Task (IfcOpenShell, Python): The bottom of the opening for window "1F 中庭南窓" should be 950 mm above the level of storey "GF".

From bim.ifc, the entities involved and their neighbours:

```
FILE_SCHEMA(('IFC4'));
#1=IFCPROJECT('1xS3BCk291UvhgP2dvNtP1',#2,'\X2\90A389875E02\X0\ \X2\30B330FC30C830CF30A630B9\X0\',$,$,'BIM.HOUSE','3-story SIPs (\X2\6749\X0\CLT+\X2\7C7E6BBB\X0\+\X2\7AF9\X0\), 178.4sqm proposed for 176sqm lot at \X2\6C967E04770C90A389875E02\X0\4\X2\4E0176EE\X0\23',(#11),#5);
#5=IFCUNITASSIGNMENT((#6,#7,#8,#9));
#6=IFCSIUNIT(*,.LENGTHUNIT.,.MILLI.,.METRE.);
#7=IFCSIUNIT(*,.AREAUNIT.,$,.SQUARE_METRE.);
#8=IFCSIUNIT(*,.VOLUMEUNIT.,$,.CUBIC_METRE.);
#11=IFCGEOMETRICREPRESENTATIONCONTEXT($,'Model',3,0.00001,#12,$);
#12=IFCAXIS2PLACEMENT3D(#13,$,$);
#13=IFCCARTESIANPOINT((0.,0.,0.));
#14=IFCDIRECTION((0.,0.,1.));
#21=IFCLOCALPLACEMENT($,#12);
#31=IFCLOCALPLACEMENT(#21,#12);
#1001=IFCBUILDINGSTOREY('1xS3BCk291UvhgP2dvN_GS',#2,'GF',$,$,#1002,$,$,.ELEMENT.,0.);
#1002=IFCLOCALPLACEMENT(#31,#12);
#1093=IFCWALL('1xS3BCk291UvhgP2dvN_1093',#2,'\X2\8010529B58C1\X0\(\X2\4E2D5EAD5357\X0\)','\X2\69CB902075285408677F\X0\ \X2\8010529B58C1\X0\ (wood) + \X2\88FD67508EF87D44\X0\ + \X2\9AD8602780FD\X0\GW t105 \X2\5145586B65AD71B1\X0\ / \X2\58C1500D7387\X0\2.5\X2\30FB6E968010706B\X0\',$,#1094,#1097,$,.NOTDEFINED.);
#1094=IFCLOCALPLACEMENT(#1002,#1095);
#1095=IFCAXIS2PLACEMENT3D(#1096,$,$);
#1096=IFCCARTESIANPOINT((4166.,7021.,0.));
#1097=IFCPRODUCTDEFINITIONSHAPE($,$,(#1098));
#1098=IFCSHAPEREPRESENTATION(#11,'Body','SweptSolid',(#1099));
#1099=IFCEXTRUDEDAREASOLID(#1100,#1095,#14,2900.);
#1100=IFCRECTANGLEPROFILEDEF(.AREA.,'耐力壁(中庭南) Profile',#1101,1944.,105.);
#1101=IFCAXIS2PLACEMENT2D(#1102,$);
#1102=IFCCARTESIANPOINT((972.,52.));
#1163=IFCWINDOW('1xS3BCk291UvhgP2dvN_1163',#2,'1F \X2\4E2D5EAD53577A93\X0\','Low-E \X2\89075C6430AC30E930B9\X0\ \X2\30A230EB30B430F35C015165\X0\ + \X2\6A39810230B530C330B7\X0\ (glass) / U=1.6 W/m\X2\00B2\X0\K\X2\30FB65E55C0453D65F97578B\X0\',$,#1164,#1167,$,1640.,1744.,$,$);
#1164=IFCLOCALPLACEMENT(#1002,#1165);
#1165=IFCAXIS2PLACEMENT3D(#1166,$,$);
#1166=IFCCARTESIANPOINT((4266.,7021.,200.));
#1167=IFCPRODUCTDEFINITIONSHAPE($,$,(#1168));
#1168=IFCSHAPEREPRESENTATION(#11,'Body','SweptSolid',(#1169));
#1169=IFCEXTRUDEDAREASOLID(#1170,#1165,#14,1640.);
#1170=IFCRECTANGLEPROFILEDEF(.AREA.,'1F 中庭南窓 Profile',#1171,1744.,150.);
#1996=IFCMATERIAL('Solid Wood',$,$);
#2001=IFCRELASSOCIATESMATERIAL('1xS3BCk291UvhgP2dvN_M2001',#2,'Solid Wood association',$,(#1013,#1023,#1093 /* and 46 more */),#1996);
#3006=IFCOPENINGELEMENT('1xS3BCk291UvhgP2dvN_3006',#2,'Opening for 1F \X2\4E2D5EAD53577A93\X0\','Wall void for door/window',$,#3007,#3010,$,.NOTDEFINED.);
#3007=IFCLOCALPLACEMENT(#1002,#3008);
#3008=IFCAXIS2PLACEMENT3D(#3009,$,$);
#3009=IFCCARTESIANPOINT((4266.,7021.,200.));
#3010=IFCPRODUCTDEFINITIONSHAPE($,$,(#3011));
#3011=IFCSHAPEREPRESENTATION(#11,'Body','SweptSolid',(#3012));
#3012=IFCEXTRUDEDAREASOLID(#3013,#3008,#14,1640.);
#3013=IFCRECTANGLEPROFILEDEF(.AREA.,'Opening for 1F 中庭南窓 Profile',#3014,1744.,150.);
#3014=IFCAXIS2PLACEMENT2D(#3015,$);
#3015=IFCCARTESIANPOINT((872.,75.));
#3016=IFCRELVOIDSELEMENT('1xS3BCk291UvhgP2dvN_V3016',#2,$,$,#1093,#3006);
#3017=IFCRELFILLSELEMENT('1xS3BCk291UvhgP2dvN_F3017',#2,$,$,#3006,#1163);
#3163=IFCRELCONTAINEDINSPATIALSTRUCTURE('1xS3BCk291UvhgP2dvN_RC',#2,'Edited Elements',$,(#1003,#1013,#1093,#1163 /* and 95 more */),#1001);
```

```python
import numpy as np
import ifcopenshell
import ifcopenshell.api.geometry
import ifcopenshell.geom
import ifcopenshell.util.element
import ifcopenshell.util.placement
import ifcopenshell.util.shape
import ifcopenshell.util.unit

model = ifcopenshell.open("bim.ifc")
unit_scale = ifcopenshell.util.unit.calculate_unit_scale(model)

window = model.by_guid("1xS3BCk291UvhgP2dvN_1163")
opening = window.FillsVoids[0].RelatingOpeningElement
storey = ifcopenshell.util.element.get_container(window, ifc_class="IfcBuildingStorey")
level = ifcopenshell.util.placement.get_local_placement(storey.ObjectPlacement)[2, 3]

# The opening's origin need not be at the sill, so measure its lowest point.
shape = ifcopenshell.geom.create_shape(ifcopenshell.geom.settings(), opening)
bottom = ifcopenshell.util.shape.get_shape_bottom_elevation(shape, shape.geometry) / unit_scale
dz = level + 0.95 / unit_scale - bottom

shift = np.array([0.0, 0.0, dz])
# The window is not placed relative to its opening, so move both.
for product in (opening, window):
    matrix = ifcopenshell.util.placement.get_local_placement(product.ObjectPlacement)
    matrix[:3, 3] += shift
    ifcopenshell.api.geometry.edit_object_placement(model, product=product, matrix=matrix, is_si=False)

print(f"moved by {dz * unit_scale:+.3f} m")

model.write("bim-out.ifc")
```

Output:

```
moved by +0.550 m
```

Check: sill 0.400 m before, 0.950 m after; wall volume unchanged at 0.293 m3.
